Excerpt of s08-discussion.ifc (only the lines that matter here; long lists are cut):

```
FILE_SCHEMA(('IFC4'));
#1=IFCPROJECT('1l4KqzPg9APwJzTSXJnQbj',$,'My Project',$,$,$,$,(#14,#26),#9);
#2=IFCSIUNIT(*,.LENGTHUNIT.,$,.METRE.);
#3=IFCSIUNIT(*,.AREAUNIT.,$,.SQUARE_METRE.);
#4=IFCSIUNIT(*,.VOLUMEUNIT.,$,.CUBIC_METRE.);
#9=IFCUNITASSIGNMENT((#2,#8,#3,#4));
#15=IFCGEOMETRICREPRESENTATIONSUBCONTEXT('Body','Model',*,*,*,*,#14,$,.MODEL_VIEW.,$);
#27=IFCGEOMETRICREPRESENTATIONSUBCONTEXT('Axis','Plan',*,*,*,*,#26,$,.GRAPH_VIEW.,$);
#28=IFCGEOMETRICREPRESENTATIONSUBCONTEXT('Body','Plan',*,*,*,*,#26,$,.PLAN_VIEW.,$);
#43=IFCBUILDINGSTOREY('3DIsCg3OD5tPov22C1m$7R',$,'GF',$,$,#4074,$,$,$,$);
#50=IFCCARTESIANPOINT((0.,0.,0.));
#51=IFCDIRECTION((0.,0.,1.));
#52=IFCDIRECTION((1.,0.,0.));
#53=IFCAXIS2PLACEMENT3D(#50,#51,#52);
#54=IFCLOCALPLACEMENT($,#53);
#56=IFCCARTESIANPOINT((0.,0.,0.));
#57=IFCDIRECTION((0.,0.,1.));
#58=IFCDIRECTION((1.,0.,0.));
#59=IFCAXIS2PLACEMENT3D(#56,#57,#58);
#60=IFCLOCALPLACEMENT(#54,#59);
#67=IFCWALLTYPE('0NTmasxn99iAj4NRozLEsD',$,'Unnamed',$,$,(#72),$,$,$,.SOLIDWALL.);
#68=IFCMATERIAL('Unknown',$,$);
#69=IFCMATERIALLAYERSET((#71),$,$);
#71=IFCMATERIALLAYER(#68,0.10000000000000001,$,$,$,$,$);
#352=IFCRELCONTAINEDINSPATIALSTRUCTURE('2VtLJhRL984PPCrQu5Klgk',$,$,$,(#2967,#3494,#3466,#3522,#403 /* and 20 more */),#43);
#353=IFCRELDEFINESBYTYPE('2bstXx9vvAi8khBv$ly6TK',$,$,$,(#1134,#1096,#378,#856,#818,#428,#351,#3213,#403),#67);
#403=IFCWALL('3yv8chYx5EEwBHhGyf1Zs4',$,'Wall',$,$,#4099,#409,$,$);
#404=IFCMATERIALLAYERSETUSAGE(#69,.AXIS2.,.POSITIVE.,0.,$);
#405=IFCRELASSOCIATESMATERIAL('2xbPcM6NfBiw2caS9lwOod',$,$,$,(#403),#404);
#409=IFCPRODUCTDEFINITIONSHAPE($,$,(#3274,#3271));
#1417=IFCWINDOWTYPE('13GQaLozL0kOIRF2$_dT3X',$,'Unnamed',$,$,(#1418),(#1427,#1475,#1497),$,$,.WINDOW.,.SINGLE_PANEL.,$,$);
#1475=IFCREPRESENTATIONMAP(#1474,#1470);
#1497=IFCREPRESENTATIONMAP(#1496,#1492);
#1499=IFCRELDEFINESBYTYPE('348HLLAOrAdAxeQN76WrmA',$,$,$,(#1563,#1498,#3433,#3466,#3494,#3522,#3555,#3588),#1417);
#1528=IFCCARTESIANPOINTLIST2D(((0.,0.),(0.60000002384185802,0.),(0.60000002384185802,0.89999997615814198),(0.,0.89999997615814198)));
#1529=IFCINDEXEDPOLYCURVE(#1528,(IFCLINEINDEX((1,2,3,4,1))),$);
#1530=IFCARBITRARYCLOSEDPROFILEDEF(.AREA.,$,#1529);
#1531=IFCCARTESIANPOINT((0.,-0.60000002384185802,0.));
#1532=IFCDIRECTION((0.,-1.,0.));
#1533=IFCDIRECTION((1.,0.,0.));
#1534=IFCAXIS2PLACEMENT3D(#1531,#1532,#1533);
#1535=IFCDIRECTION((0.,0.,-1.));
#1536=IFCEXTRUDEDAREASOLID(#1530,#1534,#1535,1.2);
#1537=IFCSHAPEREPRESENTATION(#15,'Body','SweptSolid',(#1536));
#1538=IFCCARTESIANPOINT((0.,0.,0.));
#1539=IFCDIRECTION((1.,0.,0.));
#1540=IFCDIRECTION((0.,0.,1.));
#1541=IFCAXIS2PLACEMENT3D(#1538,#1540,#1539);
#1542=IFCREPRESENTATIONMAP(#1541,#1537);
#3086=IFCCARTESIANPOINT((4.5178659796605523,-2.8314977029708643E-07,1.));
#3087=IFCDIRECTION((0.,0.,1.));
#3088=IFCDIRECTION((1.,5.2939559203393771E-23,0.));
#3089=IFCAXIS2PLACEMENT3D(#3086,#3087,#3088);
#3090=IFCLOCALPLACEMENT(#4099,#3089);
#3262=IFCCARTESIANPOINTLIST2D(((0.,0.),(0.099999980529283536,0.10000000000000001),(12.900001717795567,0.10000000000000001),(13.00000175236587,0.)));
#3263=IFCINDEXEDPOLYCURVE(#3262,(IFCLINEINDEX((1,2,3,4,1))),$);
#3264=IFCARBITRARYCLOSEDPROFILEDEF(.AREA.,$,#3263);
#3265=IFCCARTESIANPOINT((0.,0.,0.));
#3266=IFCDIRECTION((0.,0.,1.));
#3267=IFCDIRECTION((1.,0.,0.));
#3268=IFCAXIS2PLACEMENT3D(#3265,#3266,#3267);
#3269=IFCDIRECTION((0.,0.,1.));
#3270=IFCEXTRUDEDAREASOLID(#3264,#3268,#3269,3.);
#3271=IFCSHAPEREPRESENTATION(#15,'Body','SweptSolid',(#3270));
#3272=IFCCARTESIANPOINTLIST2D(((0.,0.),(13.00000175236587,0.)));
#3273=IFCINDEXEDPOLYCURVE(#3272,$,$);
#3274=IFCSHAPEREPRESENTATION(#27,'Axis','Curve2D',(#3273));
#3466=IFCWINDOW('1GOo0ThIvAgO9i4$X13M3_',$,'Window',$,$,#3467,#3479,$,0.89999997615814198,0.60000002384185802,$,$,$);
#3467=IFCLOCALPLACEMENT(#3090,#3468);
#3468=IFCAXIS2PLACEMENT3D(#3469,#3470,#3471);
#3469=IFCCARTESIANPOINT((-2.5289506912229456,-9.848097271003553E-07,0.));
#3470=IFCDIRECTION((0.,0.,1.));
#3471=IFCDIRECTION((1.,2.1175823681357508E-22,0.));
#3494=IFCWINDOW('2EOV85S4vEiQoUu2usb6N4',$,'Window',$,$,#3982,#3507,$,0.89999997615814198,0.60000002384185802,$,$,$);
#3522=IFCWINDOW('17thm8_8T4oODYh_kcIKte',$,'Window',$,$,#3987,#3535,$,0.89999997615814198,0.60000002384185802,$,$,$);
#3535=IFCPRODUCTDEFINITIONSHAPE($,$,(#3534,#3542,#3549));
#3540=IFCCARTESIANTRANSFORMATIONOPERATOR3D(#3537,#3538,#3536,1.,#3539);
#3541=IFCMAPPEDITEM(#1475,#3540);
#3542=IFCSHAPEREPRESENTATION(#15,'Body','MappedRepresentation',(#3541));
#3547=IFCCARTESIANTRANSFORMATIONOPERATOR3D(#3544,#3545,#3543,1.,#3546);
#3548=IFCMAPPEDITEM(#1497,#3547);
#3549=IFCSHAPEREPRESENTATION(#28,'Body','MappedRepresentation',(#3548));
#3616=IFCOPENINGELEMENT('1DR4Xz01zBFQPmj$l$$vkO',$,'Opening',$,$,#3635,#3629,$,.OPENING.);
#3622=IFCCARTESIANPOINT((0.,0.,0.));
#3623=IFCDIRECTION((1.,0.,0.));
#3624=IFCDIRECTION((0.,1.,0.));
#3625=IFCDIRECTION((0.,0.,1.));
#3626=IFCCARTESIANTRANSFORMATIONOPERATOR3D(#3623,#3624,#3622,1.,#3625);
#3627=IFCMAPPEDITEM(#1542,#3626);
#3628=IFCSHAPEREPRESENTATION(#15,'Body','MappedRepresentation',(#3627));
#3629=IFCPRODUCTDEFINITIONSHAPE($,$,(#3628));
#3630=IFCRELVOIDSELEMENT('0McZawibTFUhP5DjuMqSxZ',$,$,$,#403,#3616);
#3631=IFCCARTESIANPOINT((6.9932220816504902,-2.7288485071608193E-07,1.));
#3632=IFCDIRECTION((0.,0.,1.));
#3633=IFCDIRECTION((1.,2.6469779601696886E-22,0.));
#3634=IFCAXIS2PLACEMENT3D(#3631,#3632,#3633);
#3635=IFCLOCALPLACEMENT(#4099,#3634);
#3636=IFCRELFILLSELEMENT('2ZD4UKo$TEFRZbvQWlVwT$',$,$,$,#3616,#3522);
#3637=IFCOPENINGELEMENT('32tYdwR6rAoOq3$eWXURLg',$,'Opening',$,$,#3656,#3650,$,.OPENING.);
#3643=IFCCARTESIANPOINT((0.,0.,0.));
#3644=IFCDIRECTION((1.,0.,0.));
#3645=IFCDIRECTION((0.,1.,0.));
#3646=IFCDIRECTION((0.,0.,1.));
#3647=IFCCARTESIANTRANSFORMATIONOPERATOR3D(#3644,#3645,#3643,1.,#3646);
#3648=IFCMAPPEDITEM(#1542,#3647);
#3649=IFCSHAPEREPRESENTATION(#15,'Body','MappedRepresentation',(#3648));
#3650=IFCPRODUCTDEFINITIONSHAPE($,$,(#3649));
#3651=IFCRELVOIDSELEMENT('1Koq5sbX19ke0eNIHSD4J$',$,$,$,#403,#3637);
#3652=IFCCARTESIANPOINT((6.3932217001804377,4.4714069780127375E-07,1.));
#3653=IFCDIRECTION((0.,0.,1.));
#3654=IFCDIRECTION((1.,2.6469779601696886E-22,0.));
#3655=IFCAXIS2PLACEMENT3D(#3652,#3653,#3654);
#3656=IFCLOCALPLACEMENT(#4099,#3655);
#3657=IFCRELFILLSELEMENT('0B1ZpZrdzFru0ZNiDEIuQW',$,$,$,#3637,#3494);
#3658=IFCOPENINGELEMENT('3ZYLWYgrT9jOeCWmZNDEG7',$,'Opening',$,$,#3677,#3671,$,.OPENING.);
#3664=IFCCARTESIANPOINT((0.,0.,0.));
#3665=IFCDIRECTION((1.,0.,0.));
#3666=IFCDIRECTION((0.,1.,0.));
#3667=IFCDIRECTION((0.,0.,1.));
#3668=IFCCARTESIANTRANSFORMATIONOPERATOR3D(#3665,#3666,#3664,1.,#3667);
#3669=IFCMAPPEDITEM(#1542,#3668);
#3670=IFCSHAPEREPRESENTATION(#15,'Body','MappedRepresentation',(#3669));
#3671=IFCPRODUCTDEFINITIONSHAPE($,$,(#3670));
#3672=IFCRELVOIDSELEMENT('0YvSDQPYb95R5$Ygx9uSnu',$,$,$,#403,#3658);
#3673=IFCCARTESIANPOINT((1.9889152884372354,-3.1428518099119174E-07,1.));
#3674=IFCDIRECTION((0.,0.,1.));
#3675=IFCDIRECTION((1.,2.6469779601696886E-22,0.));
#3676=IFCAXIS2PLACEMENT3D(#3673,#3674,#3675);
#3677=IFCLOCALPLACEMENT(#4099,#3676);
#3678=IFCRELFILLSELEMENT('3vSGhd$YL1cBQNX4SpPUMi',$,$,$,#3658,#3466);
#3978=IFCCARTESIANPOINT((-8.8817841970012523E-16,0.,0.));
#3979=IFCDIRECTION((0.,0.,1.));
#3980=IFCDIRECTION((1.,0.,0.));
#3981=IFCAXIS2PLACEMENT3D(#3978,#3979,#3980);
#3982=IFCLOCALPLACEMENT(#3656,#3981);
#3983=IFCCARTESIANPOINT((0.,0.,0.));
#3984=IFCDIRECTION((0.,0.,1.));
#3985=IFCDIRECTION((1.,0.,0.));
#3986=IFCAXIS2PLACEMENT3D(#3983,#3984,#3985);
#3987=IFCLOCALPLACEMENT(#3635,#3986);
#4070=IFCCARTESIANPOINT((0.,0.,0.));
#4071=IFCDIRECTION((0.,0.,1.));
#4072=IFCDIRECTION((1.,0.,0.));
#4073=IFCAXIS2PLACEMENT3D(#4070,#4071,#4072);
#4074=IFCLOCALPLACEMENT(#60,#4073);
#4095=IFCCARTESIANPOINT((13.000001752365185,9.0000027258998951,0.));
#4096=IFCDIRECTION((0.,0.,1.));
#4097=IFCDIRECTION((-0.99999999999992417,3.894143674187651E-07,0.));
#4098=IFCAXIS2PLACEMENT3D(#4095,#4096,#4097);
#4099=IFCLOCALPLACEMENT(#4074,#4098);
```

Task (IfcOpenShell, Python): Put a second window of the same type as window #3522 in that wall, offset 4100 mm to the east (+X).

```python
import ifcopenshell
import ifcopenshell.api.feature
import ifcopenshell.api.geometry
import ifcopenshell.api.root
import ifcopenshell.geom
import ifcopenshell.util.element
import ifcopenshell.util.placement
import ifcopenshell.util.shape

model = ifcopenshell.open("s08-discussion.ifc")
settings = ifcopenshell.geom.settings()


def volume(element):
    """Net volume in cubic metres, openings subtracted."""
    shape = ifcopenshell.geom.create_shape(settings, element)
    return ifcopenshell.util.shape.get_volume(shape.geometry)


window = model.by_id(3522)
opening = window.FillsVoids[0].RelatingOpeningElement
wall = opening.VoidsElements[0].RelatingBuildingElement
before = volume(wall)
shift = ifcopenshell.util.placement.get_local_placement(wall.ObjectPlacement)[:3, 0] * -4.1

# copy_class copies the void relationship, type, container and properties, but no geometry.
new_opening = ifcopenshell.api.root.copy_class(model, product=opening)
new_opening.Representation = ifcopenshell.util.element.copy_deep(
    model, opening.Representation, exclude=["IfcGeometricRepresentationContext", "IfcRepresentationMap"]
)
new_window = ifcopenshell.api.root.copy_class(model, product=window)
new_window.Representation = ifcopenshell.util.element.copy_deep(
    model, window.Representation, exclude=["IfcGeometricRepresentationContext", "IfcRepresentationMap"]
)
ifcopenshell.api.feature.add_filling(model, opening=new_opening, element=new_window)

for old, new in ((opening, new_opening), (window, new_window)):
    matrix = ifcopenshell.util.placement.get_local_placement(old.ObjectPlacement)
    matrix[:3, 3] += shift
    ifcopenshell.api.geometry.edit_object_placement(model, product=new, matrix=matrix, is_si=False)

after = volume(wall)

print(f"wall volume {before:.3f} -> {after:.3f} m3")

model.write("s08-discussion_v2.ifc")
```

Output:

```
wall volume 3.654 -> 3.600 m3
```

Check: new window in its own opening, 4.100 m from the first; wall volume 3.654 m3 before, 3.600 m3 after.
